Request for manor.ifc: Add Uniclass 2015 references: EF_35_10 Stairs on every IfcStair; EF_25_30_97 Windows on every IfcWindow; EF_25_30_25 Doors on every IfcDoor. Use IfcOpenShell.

First a look at what the model holds.

```python
import ifcopenshell

model = ifcopenshell.open("manor.ifc")
print(model.schema)
print("classifications:", [c.Name for c in model.by_type("IfcClassification")])
for ifc_class in ("IfcDoor", "IfcRoof", "IfcStair", "IfcWall", "IfcWindow"):
    print(ifc_class, len(model.by_type(ifc_class)))
```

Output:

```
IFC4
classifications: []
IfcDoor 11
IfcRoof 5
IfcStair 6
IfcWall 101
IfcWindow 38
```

```python
import ifcopenshell
import ifcopenshell.api.classification

model = ifcopenshell.open("manor.ifc")

system = ifcopenshell.api.classification.add_classification(model, classification="Uniclass 2015")

codes = {
    "IfcStair": ("EF_35_10", "Stairs"),
    "IfcWindow": ("EF_25_30_97", "Windows"),
    "IfcDoor": ("EF_25_30_25", "Doors"),
}
for ifc_class, (code, name) in codes.items():
    products = model.by_type(ifc_class)
    ifcopenshell.api.classification.add_reference(
        model, products=products, classification=system, identification=code, name=name
    )
    print(code, len(products))

model.write("manor_updated.ifc")
```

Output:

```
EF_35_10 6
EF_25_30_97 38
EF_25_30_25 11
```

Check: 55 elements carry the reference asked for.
